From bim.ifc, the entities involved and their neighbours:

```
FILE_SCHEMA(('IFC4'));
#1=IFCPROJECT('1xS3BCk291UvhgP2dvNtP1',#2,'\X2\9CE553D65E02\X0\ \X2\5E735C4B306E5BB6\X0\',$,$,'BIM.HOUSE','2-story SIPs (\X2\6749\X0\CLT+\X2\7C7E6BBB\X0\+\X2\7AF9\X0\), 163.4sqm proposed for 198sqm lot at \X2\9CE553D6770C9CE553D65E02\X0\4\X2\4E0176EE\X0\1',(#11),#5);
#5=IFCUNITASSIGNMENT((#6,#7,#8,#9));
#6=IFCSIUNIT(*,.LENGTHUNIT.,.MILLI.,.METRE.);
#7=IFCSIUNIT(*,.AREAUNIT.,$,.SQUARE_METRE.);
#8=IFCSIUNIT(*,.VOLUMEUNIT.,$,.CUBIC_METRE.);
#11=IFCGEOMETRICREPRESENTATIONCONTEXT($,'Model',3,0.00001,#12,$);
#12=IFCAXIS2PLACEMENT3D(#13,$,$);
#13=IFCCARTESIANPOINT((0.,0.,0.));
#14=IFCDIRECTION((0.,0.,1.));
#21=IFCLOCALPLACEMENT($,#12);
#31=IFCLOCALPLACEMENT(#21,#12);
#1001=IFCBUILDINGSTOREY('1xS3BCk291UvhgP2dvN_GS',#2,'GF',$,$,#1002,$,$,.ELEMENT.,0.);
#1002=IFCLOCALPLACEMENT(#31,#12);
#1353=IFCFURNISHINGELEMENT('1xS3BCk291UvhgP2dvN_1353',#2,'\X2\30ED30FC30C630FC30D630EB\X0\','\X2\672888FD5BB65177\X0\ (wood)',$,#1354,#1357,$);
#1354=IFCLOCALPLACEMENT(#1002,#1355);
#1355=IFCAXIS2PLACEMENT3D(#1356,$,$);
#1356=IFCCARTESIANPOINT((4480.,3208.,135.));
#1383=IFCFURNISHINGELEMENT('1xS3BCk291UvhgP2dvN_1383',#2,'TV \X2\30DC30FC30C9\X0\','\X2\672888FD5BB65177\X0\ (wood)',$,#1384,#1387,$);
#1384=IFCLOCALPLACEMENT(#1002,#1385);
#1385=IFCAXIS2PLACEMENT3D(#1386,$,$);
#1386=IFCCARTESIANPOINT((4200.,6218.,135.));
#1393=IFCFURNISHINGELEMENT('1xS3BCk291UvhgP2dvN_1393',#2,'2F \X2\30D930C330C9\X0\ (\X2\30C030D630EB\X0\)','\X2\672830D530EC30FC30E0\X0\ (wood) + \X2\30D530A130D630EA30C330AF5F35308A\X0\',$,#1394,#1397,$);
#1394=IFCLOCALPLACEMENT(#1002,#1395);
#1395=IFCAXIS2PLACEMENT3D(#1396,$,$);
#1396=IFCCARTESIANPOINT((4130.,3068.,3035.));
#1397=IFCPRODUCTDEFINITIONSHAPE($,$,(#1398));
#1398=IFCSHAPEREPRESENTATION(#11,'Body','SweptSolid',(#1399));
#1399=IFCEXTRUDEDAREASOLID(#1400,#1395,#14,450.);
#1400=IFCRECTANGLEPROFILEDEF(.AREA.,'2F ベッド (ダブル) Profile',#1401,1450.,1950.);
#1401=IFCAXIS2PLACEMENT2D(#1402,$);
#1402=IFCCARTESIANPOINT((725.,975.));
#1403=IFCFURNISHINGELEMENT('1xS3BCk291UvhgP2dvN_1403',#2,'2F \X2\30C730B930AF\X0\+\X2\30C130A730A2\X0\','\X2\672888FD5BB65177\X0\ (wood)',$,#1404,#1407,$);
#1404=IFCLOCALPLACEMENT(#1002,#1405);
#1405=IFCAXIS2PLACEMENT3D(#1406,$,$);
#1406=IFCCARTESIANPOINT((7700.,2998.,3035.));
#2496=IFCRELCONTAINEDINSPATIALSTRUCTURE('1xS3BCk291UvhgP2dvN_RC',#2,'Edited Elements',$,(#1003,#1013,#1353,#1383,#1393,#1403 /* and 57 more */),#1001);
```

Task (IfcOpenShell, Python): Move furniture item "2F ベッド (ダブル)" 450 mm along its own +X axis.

```python
import ifcopenshell
import ifcopenshell.api.geometry
import ifcopenshell.util.placement
import ifcopenshell.util.unit

model = ifcopenshell.open("bim.ifc")
unit_scale = ifcopenshell.util.unit.calculate_unit_scale(model)

item = model.by_id(1393)
matrix = ifcopenshell.util.placement.get_local_placement(item.ObjectPlacement)
matrix[:3, 3] += matrix[:3, 0] * 0.45 / unit_scale
ifcopenshell.api.geometry.edit_object_placement(model, product=item, matrix=matrix, is_si=False)

print(ifcopenshell.util.placement.get_local_placement(item.ObjectPlacement).round(3) + 0.0)

model.write("bim-out.ifc")
```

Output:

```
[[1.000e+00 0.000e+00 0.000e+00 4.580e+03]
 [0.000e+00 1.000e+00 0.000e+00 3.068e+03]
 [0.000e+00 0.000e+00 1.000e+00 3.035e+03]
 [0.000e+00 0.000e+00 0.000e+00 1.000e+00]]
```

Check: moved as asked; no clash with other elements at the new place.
